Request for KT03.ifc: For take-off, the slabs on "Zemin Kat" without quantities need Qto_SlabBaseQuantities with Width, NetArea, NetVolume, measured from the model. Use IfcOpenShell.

First a look at what the model holds.

```python
import ifcopenshell
import ifcopenshell.util.element
import ifcopenshell.util.unit

model = ifcopenshell.open("KT03.ifc")
print(model.schema)
for unit_type in ("LENGTHUNIT", "AREAUNIT", "VOLUMEUNIT"):
    print(unit_type, ifcopenshell.util.unit.calculate_unit_scale(model, unit_type))
storey = next(s for s in model.by_type("IfcBuildingStorey") if s.Name == "Zemin Kat")
slabs = [e for e in ifcopenshell.util.element.get_decomposition(storey) if e.is_a("IfcSlab")]
for e in sorted(slabs, key=lambda e: e.id()):
    print(e.id(), e.is_a(), e.Name, list(ifcopenshell.util.element.get_psets(e, qtos_only=True)), sep=" | ")
```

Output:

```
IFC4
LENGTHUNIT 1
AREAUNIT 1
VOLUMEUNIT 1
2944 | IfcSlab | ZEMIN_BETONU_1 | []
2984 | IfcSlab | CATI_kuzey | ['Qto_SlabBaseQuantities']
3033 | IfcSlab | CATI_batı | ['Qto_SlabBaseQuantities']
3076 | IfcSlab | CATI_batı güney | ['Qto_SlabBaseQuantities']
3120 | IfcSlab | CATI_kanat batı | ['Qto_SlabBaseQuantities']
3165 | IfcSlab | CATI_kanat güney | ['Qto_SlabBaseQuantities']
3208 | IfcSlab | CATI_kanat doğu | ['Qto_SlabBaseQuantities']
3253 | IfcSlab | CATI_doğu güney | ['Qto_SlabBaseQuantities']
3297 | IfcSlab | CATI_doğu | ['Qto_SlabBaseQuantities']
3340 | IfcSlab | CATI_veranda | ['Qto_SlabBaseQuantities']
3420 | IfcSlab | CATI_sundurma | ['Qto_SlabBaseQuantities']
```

```python
import ifcopenshell
import ifcopenshell.api.pset
import ifcopenshell.geom
import ifcopenshell.util.element
import ifcopenshell.util.shape
import ifcopenshell.util.unit

model = ifcopenshell.open("KT03.ifc")
unit_scale = ifcopenshell.util.unit.calculate_unit_scale(model)
area_scale = ifcopenshell.util.unit.calculate_unit_scale(model, "AREAUNIT")
volume_scale = ifcopenshell.util.unit.calculate_unit_scale(model, "VOLUMEUNIT")
settings = ifcopenshell.geom.settings()

storey = next(s for s in model.by_type("IfcBuildingStorey") if s.Name == "Zemin Kat")
slabs = [e for e in ifcopenshell.util.element.get_decomposition(storey) if e.is_a("IfcSlab")]

for e in sorted(slabs, key=lambda e: e.id()):
    if ifcopenshell.util.element.get_psets(e, qtos_only=True, should_inherit=False):
        continue
    # Geometry comes back in metres, in the element's own axes.
    shape = ifcopenshell.geom.create_shape(settings, e)
    values = {
        "Width": ifcopenshell.util.shape.get_z(shape.geometry) / unit_scale,
        "NetArea": ifcopenshell.util.shape.get_footprint_area(shape.geometry) / area_scale,
        "NetVolume": ifcopenshell.util.shape.get_volume(shape.geometry) / volume_scale,
    }
    qto = ifcopenshell.api.pset.add_qto(model, product=e, name="Qto_SlabBaseQuantities")
    ifcopenshell.api.pset.edit_qto(model, qto=qto, properties=values)
    print(e.id(), {k: round(v, 3) for k, v in values.items()})

model.write("KT03_edited.ifc")
```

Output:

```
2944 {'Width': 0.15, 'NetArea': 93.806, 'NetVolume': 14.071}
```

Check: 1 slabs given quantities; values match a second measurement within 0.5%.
